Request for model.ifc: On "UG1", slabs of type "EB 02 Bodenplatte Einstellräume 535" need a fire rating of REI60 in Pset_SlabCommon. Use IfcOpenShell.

First a look at what the model holds.

```python
import ifcopenshell
import ifcopenshell.util.element

model = ifcopenshell.open("model.ifc")
print(model.schema)
storey = next(s for s in model.by_type("IfcBuildingStorey") if s.Name == "UG1")
slabs = [e for e in ifcopenshell.util.element.get_decomposition(storey) if e.is_a("IfcSlab")]
seen = {}
for e in slabs:
    element_type = ifcopenshell.util.element.get_type(e)
    key = (element_type.Name if element_type != e and element_type else None, ifcopenshell.util.element.get_pset(e, "Pset_SlabCommon", "FireRating"))
    seen[key] = seen.get(key, 0) + 1
for (name, value), count in sorted(seen.items(), key=str):
    print(count, "x", name, "|", value)
```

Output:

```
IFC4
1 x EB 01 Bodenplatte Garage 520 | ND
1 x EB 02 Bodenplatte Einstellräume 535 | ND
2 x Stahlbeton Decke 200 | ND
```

```python
import ifcopenshell
import ifcopenshell.api.pset
import ifcopenshell.util.element

model = ifcopenshell.open("model.ifc")

storey = next(s for s in model.by_type("IfcBuildingStorey") if s.Name == "UG1")
slabs = [e for e in ifcopenshell.util.element.get_decomposition(storey) if e.is_a("IfcSlab")]

count = 0
for e in slabs:
    element_type = ifcopenshell.util.element.get_type(e)
    if element_type in (None, e) or element_type.Name != "EB 02 Bodenplatte Einstellräume 535":
        continue
    # add_pset returns the element's existing set when there is one.
    pset = ifcopenshell.api.pset.add_pset(model, product=e, name="Pset_SlabCommon")
    ifcopenshell.api.pset.edit_pset(model, pset=pset, properties={"FireRating": "REI60"})
    count += 1

print(count, "slabs updated")

model.write("model_rev.ifc")
```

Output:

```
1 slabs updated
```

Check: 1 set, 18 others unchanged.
